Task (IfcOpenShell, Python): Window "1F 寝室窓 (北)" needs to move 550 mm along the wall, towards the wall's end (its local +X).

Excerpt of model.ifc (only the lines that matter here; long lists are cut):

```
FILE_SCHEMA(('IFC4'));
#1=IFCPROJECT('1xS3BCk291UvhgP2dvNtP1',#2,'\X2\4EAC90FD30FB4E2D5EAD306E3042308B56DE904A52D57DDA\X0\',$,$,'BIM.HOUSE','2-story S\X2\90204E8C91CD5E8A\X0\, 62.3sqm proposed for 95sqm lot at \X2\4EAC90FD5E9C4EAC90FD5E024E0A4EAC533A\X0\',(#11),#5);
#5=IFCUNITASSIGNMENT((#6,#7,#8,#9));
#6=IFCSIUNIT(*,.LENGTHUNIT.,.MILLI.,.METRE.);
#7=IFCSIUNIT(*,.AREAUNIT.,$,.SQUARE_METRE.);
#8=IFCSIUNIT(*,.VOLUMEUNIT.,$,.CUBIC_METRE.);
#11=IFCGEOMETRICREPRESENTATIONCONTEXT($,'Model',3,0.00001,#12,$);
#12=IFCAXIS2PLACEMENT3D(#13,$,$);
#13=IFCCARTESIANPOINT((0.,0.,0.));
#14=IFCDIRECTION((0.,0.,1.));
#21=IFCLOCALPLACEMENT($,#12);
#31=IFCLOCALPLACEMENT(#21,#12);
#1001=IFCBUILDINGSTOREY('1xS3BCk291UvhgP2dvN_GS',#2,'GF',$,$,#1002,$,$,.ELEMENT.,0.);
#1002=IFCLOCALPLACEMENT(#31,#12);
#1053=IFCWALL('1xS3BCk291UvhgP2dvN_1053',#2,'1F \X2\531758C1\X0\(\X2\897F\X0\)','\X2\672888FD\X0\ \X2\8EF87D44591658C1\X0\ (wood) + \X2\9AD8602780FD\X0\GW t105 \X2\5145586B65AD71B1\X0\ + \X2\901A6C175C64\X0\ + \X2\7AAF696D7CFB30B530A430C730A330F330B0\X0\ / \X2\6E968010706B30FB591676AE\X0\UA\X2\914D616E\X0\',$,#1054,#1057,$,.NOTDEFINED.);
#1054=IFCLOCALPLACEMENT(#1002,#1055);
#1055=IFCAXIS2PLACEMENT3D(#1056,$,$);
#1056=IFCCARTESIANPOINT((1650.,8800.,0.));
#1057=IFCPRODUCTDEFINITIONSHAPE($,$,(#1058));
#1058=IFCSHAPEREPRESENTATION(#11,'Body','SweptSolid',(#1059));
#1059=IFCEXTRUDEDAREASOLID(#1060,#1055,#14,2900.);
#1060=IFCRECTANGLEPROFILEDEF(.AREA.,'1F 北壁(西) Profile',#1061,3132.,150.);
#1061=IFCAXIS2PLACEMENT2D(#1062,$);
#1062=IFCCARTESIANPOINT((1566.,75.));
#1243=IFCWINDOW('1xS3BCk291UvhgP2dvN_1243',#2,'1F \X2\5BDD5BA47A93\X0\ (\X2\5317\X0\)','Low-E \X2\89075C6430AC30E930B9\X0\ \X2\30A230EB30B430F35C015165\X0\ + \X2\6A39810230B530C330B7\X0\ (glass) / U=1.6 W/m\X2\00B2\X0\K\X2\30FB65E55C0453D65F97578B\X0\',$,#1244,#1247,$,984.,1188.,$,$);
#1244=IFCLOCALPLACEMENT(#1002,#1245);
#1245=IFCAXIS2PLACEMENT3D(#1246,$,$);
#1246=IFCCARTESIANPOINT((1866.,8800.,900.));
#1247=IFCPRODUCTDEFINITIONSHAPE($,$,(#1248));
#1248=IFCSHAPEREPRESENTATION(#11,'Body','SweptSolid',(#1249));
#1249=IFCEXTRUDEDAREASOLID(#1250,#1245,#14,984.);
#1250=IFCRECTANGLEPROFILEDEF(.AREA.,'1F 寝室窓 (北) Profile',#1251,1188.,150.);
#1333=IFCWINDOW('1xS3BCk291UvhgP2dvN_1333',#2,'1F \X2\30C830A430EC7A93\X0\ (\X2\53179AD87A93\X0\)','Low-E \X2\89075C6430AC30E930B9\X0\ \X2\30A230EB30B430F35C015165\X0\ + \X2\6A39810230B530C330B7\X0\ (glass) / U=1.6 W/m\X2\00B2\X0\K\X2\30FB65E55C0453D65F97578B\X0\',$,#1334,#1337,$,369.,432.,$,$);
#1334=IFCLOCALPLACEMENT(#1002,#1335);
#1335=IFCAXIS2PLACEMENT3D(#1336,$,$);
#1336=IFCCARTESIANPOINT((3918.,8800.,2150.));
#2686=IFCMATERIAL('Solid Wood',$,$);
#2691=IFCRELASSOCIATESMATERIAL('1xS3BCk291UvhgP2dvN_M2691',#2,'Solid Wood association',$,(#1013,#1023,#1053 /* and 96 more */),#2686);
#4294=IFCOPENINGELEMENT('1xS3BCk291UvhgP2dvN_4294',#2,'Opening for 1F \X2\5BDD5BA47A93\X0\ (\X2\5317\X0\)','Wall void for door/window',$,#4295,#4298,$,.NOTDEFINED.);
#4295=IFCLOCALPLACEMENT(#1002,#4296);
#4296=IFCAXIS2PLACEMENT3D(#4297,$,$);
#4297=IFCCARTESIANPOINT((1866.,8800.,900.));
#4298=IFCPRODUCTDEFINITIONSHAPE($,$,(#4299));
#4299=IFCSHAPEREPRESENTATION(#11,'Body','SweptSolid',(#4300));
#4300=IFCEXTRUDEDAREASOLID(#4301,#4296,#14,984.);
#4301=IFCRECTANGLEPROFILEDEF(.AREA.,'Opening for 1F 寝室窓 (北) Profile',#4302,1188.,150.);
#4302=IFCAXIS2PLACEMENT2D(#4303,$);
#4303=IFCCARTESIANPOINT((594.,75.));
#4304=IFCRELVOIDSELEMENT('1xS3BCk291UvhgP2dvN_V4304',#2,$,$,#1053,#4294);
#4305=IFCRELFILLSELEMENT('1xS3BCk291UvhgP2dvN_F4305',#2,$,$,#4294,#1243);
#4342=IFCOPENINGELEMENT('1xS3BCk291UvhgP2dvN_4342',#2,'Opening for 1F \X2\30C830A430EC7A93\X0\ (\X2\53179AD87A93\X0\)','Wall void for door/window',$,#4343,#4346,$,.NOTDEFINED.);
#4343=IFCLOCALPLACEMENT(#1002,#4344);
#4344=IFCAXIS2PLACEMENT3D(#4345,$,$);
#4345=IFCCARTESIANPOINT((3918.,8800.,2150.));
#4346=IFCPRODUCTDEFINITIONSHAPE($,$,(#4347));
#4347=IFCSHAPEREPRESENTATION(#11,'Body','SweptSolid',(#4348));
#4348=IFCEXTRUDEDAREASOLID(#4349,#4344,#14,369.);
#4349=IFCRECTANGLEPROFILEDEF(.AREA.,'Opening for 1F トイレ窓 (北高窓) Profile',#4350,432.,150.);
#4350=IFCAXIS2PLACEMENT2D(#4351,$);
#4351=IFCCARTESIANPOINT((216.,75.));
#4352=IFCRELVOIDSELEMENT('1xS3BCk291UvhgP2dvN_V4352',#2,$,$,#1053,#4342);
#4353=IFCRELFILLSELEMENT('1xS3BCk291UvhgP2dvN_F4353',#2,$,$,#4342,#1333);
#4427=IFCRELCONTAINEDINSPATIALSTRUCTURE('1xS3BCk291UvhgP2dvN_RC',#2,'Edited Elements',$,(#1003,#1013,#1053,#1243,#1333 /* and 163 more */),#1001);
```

```python
import ifcopenshell
import ifcopenshell.api.geometry
import ifcopenshell.util.placement
import ifcopenshell.util.unit

model = ifcopenshell.open("model.ifc")
unit_scale = ifcopenshell.util.unit.calculate_unit_scale(model)

window = model.by_guid("1xS3BCk291UvhgP2dvN_1243")
opening = window.FillsVoids[0].RelatingOpeningElement
wall = opening.VoidsElements[0].RelatingBuildingElement

wall_matrix = ifcopenshell.util.placement.get_local_placement(wall.ObjectPlacement)
shift = wall_matrix[:3, 0] * 0.55 / unit_scale
before = ifcopenshell.util.placement.get_local_placement(window.ObjectPlacement)[:3, 3].copy()

# The window is not placed relative to its opening, so move both.
for product in (opening, window):
    matrix = ifcopenshell.util.placement.get_local_placement(product.ObjectPlacement)
    matrix[:3, 3] += shift
    ifcopenshell.api.geometry.edit_object_placement(model, product=product, matrix=matrix, is_si=False)

after = ifcopenshell.util.placement.get_local_placement(window.ObjectPlacement)[:3, 3]
print("window moved by", (after - before).round(3) + 0.0)

model.write("model_edited.ifc")
```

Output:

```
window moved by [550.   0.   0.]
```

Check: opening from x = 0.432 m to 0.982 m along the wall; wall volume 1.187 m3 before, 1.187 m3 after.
